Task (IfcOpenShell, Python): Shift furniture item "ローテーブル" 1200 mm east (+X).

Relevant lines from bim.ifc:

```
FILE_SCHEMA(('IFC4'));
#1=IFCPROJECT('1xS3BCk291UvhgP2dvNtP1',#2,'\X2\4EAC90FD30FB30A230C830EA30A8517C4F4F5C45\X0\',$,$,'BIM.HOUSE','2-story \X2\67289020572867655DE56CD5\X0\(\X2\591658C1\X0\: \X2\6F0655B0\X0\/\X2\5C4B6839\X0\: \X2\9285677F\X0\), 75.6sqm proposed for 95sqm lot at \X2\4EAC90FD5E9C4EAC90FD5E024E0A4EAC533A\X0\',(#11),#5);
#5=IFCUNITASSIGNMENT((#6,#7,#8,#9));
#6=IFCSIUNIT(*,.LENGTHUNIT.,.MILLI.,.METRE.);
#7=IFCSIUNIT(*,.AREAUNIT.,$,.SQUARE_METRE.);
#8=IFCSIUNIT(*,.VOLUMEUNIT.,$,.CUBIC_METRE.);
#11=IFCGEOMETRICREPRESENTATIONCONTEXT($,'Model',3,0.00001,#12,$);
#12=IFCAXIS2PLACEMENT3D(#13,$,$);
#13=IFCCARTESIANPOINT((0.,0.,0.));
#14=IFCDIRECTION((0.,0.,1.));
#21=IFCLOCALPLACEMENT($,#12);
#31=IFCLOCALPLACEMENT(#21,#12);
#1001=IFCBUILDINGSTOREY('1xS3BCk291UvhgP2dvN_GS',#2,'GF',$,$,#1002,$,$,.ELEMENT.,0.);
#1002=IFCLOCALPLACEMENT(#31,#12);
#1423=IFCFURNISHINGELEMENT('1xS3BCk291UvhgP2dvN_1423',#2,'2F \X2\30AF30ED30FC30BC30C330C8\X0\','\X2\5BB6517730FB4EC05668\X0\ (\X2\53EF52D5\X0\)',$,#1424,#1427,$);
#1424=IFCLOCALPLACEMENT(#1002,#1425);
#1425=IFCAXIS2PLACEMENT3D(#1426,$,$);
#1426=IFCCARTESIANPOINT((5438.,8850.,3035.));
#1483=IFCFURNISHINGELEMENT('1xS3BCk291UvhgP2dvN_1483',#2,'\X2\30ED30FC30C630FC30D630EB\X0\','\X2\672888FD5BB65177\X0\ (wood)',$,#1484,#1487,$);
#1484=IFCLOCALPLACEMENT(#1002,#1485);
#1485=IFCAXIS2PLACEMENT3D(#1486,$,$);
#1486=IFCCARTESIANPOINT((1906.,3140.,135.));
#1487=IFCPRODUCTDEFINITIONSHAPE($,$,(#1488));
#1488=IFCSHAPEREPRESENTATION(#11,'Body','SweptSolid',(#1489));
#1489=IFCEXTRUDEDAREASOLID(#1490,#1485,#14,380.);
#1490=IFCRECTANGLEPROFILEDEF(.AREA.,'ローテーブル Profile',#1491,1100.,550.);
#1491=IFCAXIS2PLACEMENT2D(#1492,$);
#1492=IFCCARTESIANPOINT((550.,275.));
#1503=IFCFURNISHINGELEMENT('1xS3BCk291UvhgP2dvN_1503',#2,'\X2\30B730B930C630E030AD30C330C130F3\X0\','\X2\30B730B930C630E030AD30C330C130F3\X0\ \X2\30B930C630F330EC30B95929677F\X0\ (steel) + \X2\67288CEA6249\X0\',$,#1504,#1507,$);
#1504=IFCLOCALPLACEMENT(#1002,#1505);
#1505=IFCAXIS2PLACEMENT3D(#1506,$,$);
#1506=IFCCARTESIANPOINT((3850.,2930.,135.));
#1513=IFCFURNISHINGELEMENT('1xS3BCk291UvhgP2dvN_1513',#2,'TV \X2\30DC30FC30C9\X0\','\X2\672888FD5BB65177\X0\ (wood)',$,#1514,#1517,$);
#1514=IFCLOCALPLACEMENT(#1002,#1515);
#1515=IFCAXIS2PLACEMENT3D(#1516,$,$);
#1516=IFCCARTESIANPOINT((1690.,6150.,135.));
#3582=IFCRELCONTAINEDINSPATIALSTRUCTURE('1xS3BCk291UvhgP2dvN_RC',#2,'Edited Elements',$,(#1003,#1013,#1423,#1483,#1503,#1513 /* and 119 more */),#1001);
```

```python
import ifcopenshell
import ifcopenshell.api.geometry
import ifcopenshell.util.placement
import ifcopenshell.util.unit

model = ifcopenshell.open("bim.ifc")
unit_scale = ifcopenshell.util.unit.calculate_unit_scale(model)

item = model.by_guid("1xS3BCk291UvhgP2dvN_1483")
matrix = ifcopenshell.util.placement.get_local_placement(item.ObjectPlacement)
matrix[0, 3] += 1.2 / unit_scale
ifcopenshell.api.geometry.edit_object_placement(model, product=item, matrix=matrix, is_si=False)

print(ifcopenshell.util.placement.get_local_placement(item.ObjectPlacement).round(3) + 0.0)

model.write("bim_rev.ifc")
```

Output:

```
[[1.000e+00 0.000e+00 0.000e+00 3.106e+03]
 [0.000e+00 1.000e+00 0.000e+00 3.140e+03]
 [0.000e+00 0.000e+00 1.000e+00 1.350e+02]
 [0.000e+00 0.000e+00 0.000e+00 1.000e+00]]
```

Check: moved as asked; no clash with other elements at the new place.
